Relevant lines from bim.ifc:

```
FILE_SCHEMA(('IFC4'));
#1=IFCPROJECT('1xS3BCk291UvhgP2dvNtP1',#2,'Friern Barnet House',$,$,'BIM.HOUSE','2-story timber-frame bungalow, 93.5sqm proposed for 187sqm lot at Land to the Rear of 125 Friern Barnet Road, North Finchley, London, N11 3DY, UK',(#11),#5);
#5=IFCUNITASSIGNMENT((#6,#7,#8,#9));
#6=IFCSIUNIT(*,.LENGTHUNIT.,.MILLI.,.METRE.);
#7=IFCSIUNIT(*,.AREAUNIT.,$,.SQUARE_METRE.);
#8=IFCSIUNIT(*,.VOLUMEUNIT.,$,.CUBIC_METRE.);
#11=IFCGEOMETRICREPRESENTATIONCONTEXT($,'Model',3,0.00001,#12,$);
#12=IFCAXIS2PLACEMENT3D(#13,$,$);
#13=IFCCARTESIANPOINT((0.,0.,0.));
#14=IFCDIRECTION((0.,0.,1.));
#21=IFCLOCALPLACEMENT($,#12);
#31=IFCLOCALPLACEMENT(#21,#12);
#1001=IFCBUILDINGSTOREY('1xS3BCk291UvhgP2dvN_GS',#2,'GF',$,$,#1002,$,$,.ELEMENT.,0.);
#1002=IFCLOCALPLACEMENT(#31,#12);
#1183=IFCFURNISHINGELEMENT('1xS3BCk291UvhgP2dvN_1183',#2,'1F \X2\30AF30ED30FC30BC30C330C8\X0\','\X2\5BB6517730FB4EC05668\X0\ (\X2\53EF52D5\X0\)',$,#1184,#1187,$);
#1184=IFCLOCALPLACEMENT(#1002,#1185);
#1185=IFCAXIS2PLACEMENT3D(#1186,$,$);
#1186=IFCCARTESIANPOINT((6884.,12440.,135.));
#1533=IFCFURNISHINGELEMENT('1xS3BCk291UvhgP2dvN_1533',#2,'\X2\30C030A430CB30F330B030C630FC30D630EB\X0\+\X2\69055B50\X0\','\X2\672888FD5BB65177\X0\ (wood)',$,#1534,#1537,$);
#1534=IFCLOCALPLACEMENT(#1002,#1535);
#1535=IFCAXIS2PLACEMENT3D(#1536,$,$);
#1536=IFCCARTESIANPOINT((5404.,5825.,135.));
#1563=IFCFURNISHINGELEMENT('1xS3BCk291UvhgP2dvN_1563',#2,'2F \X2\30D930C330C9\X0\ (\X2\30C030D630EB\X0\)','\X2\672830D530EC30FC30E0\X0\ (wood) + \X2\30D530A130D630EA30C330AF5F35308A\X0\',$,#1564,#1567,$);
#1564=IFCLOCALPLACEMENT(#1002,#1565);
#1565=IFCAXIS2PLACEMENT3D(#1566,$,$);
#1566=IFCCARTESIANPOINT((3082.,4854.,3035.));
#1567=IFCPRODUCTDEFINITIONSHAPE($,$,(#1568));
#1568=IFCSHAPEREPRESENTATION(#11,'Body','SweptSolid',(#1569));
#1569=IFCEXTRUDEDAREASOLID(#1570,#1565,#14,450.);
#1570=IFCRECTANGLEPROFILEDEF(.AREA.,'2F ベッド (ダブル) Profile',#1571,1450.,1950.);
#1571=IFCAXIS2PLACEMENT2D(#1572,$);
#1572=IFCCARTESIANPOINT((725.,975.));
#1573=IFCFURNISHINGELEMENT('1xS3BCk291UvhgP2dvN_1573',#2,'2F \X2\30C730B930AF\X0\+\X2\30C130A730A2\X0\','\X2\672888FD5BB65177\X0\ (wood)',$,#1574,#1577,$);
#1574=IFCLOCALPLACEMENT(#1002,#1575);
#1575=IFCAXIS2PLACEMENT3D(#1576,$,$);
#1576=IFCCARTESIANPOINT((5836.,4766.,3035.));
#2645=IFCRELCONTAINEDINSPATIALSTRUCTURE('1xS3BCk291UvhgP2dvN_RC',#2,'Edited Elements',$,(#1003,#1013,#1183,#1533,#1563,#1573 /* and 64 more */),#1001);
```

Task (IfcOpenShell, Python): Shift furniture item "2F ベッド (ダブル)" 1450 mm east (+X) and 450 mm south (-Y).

```python
import ifcopenshell
import ifcopenshell.api.geometry
import ifcopenshell.util.placement

model = ifcopenshell.open("bim.ifc")

item = model.by_guid("1xS3BCk291UvhgP2dvN_1563")
matrix = ifcopenshell.util.placement.get_local_placement(item.ObjectPlacement)
matrix[0, 3] += 1450.0
matrix[1, 3] -= 450.0
ifcopenshell.api.geometry.edit_object_placement(model, product=item, matrix=matrix, is_si=False)

print(ifcopenshell.util.placement.get_local_placement(item.ObjectPlacement).round(3) + 0.0)

model.write("bim_updated.ifc")
```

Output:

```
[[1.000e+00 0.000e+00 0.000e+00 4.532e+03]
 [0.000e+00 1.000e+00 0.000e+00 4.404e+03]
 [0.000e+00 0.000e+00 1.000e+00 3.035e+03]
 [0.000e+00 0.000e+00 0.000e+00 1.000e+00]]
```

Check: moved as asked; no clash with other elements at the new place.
